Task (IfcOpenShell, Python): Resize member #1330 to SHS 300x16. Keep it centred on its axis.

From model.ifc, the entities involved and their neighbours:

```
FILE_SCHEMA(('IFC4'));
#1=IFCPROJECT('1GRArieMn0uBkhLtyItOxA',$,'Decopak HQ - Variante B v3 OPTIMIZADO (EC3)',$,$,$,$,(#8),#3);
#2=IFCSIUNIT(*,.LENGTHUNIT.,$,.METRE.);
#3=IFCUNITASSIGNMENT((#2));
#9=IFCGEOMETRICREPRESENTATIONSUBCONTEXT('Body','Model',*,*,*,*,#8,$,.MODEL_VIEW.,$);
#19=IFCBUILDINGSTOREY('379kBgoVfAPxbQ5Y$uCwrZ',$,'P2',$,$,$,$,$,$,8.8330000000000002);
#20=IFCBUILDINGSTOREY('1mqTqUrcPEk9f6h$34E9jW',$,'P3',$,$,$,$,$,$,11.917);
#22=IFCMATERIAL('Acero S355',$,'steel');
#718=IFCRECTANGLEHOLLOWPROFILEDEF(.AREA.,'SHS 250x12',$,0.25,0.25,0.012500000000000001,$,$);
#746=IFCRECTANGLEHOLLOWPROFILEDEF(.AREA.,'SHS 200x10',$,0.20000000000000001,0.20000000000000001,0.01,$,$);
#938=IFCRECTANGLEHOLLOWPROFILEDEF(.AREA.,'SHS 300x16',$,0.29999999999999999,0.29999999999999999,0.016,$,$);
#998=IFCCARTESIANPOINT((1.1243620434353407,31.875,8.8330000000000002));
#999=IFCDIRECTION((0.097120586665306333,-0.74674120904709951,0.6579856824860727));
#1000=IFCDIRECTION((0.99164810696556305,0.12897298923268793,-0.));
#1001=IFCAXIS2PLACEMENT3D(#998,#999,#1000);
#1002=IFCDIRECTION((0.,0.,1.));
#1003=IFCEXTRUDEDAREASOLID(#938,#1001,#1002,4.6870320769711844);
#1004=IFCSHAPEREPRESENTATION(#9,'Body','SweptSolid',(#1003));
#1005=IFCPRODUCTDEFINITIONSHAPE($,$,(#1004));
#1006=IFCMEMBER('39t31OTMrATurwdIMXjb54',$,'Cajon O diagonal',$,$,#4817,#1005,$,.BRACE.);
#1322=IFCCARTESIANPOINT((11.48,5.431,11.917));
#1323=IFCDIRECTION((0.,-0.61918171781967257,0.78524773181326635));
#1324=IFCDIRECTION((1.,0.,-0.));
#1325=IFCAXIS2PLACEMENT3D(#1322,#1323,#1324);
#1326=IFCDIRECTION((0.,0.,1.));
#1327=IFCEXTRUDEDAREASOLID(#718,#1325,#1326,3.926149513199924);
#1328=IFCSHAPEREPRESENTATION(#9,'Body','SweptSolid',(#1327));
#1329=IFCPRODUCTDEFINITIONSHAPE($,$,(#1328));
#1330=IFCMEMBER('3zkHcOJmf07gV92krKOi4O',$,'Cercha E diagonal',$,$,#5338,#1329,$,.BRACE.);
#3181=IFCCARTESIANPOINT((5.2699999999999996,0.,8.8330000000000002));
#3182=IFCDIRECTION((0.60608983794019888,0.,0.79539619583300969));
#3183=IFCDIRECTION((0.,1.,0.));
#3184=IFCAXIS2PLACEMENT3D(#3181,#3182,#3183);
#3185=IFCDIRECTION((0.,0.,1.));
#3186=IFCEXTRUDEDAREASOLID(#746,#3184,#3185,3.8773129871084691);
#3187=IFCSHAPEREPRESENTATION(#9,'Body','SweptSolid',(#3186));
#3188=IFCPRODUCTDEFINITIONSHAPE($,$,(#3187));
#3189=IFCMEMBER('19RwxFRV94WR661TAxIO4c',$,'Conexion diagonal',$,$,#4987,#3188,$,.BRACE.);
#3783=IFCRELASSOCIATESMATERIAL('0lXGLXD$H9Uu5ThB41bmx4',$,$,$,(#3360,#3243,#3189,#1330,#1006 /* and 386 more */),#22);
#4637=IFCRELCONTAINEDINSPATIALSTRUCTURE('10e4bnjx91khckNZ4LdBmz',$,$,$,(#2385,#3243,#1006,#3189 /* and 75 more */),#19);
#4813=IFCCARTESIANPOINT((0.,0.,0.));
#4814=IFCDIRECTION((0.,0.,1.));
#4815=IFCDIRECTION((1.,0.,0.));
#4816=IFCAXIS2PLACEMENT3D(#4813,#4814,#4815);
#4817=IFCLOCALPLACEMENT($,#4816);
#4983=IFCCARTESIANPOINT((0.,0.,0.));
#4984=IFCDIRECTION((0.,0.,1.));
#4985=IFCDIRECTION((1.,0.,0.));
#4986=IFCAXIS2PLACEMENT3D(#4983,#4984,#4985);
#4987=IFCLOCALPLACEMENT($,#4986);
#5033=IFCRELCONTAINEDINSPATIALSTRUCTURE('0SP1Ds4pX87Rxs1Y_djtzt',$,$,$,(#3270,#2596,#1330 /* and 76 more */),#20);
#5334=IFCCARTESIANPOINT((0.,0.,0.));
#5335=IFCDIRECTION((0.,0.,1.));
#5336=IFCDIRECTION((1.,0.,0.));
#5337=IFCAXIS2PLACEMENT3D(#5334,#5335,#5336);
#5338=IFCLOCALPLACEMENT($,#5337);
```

```python
import ifcopenshell
import ifcopenshell.util.element
import ifcopenshell.util.representation

model = ifcopenshell.open("model.ifc")

member = model.by_guid("3zkHcOJmf07gV92krKOi4O")
source = next(p for p in model.by_type("IfcRectangleHollowProfileDef") if p.ProfileName == "SHS 300x16")

body = ifcopenshell.util.representation.get_representation(member, "Model", "Body")
solid = body.Items[0]
old_profile = solid.SweptArea

# Copy the section's sizes but keep this member's own profile position.
profile = ifcopenshell.util.element.copy(model, source)
profile.Position = old_profile.Position
solid.SweptArea = profile
if not model.get_total_inverses(old_profile):
    ifcopenshell.util.element.remove_deep2(model, old_profile)

print(solid.SweptArea)

model.write("model_rev.ifc")
```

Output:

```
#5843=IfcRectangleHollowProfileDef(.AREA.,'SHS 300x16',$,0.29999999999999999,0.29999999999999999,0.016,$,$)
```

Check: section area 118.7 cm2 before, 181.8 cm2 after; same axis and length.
